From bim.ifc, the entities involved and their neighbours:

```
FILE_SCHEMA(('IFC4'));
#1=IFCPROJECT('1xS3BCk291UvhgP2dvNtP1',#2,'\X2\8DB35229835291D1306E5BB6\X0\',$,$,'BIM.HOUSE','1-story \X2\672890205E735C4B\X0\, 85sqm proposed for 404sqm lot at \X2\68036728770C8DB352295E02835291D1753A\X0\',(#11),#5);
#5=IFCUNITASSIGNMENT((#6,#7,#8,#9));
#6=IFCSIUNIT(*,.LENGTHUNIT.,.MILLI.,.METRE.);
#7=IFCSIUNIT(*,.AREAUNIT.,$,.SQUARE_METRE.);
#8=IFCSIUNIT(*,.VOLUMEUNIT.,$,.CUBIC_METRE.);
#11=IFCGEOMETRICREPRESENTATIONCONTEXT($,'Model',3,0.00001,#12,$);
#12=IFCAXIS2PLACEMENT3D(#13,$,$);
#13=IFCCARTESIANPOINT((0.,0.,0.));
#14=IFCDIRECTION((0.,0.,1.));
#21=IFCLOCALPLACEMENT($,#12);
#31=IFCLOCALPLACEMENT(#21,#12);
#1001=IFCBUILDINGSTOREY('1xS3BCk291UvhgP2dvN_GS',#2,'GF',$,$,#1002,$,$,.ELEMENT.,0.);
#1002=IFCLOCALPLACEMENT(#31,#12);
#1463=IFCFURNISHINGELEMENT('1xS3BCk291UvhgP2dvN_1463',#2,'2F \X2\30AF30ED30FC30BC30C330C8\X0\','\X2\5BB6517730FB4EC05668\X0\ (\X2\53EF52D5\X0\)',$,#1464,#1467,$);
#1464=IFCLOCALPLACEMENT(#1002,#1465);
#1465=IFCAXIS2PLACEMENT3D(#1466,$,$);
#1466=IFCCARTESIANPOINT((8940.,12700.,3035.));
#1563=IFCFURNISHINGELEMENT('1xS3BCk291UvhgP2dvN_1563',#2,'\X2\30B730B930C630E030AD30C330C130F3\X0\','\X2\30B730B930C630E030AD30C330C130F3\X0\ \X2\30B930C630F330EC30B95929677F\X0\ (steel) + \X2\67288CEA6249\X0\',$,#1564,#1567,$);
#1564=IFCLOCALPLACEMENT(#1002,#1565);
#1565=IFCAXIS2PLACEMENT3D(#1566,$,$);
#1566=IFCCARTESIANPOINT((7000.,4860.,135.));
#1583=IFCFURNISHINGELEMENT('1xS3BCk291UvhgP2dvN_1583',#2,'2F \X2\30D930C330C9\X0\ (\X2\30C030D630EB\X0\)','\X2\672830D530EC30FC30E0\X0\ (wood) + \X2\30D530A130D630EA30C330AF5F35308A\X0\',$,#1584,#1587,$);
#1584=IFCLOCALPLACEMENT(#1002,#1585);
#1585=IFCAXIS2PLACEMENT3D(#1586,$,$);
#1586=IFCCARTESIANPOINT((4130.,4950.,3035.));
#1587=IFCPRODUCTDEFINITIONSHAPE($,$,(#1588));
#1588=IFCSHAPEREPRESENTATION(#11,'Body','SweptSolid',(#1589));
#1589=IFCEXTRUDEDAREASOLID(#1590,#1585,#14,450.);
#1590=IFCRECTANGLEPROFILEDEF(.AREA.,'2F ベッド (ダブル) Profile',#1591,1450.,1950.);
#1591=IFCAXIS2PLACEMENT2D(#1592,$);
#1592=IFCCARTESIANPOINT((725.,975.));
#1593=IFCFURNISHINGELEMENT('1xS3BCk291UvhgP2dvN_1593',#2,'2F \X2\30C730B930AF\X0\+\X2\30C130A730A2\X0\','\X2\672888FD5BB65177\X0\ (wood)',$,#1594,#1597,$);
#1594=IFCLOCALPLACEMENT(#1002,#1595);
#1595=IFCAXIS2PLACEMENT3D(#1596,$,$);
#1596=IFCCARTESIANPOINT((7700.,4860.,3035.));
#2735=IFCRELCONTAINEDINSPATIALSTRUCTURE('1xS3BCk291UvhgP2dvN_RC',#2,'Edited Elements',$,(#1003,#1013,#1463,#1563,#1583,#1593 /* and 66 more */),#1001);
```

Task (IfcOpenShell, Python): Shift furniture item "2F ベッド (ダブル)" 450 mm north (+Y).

```python
import ifcopenshell
import ifcopenshell.api.geometry
import ifcopenshell.util.placement
import ifcopenshell.util.unit

model = ifcopenshell.open("bim.ifc")
unit_scale = ifcopenshell.util.unit.calculate_unit_scale(model)

item = model.by_guid("1xS3BCk291UvhgP2dvN_1583")
matrix = ifcopenshell.util.placement.get_local_placement(item.ObjectPlacement)
matrix[1, 3] += 0.45 / unit_scale
ifcopenshell.api.geometry.edit_object_placement(model, product=item, matrix=matrix, is_si=False)

print(ifcopenshell.util.placement.get_local_placement(item.ObjectPlacement).round(3) + 0.0)

model.write("bim_edited.ifc")
```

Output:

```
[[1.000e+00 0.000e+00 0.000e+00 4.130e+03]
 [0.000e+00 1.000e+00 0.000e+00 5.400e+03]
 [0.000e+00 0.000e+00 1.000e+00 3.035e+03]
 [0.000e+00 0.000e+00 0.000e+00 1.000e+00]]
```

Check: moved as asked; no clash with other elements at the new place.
